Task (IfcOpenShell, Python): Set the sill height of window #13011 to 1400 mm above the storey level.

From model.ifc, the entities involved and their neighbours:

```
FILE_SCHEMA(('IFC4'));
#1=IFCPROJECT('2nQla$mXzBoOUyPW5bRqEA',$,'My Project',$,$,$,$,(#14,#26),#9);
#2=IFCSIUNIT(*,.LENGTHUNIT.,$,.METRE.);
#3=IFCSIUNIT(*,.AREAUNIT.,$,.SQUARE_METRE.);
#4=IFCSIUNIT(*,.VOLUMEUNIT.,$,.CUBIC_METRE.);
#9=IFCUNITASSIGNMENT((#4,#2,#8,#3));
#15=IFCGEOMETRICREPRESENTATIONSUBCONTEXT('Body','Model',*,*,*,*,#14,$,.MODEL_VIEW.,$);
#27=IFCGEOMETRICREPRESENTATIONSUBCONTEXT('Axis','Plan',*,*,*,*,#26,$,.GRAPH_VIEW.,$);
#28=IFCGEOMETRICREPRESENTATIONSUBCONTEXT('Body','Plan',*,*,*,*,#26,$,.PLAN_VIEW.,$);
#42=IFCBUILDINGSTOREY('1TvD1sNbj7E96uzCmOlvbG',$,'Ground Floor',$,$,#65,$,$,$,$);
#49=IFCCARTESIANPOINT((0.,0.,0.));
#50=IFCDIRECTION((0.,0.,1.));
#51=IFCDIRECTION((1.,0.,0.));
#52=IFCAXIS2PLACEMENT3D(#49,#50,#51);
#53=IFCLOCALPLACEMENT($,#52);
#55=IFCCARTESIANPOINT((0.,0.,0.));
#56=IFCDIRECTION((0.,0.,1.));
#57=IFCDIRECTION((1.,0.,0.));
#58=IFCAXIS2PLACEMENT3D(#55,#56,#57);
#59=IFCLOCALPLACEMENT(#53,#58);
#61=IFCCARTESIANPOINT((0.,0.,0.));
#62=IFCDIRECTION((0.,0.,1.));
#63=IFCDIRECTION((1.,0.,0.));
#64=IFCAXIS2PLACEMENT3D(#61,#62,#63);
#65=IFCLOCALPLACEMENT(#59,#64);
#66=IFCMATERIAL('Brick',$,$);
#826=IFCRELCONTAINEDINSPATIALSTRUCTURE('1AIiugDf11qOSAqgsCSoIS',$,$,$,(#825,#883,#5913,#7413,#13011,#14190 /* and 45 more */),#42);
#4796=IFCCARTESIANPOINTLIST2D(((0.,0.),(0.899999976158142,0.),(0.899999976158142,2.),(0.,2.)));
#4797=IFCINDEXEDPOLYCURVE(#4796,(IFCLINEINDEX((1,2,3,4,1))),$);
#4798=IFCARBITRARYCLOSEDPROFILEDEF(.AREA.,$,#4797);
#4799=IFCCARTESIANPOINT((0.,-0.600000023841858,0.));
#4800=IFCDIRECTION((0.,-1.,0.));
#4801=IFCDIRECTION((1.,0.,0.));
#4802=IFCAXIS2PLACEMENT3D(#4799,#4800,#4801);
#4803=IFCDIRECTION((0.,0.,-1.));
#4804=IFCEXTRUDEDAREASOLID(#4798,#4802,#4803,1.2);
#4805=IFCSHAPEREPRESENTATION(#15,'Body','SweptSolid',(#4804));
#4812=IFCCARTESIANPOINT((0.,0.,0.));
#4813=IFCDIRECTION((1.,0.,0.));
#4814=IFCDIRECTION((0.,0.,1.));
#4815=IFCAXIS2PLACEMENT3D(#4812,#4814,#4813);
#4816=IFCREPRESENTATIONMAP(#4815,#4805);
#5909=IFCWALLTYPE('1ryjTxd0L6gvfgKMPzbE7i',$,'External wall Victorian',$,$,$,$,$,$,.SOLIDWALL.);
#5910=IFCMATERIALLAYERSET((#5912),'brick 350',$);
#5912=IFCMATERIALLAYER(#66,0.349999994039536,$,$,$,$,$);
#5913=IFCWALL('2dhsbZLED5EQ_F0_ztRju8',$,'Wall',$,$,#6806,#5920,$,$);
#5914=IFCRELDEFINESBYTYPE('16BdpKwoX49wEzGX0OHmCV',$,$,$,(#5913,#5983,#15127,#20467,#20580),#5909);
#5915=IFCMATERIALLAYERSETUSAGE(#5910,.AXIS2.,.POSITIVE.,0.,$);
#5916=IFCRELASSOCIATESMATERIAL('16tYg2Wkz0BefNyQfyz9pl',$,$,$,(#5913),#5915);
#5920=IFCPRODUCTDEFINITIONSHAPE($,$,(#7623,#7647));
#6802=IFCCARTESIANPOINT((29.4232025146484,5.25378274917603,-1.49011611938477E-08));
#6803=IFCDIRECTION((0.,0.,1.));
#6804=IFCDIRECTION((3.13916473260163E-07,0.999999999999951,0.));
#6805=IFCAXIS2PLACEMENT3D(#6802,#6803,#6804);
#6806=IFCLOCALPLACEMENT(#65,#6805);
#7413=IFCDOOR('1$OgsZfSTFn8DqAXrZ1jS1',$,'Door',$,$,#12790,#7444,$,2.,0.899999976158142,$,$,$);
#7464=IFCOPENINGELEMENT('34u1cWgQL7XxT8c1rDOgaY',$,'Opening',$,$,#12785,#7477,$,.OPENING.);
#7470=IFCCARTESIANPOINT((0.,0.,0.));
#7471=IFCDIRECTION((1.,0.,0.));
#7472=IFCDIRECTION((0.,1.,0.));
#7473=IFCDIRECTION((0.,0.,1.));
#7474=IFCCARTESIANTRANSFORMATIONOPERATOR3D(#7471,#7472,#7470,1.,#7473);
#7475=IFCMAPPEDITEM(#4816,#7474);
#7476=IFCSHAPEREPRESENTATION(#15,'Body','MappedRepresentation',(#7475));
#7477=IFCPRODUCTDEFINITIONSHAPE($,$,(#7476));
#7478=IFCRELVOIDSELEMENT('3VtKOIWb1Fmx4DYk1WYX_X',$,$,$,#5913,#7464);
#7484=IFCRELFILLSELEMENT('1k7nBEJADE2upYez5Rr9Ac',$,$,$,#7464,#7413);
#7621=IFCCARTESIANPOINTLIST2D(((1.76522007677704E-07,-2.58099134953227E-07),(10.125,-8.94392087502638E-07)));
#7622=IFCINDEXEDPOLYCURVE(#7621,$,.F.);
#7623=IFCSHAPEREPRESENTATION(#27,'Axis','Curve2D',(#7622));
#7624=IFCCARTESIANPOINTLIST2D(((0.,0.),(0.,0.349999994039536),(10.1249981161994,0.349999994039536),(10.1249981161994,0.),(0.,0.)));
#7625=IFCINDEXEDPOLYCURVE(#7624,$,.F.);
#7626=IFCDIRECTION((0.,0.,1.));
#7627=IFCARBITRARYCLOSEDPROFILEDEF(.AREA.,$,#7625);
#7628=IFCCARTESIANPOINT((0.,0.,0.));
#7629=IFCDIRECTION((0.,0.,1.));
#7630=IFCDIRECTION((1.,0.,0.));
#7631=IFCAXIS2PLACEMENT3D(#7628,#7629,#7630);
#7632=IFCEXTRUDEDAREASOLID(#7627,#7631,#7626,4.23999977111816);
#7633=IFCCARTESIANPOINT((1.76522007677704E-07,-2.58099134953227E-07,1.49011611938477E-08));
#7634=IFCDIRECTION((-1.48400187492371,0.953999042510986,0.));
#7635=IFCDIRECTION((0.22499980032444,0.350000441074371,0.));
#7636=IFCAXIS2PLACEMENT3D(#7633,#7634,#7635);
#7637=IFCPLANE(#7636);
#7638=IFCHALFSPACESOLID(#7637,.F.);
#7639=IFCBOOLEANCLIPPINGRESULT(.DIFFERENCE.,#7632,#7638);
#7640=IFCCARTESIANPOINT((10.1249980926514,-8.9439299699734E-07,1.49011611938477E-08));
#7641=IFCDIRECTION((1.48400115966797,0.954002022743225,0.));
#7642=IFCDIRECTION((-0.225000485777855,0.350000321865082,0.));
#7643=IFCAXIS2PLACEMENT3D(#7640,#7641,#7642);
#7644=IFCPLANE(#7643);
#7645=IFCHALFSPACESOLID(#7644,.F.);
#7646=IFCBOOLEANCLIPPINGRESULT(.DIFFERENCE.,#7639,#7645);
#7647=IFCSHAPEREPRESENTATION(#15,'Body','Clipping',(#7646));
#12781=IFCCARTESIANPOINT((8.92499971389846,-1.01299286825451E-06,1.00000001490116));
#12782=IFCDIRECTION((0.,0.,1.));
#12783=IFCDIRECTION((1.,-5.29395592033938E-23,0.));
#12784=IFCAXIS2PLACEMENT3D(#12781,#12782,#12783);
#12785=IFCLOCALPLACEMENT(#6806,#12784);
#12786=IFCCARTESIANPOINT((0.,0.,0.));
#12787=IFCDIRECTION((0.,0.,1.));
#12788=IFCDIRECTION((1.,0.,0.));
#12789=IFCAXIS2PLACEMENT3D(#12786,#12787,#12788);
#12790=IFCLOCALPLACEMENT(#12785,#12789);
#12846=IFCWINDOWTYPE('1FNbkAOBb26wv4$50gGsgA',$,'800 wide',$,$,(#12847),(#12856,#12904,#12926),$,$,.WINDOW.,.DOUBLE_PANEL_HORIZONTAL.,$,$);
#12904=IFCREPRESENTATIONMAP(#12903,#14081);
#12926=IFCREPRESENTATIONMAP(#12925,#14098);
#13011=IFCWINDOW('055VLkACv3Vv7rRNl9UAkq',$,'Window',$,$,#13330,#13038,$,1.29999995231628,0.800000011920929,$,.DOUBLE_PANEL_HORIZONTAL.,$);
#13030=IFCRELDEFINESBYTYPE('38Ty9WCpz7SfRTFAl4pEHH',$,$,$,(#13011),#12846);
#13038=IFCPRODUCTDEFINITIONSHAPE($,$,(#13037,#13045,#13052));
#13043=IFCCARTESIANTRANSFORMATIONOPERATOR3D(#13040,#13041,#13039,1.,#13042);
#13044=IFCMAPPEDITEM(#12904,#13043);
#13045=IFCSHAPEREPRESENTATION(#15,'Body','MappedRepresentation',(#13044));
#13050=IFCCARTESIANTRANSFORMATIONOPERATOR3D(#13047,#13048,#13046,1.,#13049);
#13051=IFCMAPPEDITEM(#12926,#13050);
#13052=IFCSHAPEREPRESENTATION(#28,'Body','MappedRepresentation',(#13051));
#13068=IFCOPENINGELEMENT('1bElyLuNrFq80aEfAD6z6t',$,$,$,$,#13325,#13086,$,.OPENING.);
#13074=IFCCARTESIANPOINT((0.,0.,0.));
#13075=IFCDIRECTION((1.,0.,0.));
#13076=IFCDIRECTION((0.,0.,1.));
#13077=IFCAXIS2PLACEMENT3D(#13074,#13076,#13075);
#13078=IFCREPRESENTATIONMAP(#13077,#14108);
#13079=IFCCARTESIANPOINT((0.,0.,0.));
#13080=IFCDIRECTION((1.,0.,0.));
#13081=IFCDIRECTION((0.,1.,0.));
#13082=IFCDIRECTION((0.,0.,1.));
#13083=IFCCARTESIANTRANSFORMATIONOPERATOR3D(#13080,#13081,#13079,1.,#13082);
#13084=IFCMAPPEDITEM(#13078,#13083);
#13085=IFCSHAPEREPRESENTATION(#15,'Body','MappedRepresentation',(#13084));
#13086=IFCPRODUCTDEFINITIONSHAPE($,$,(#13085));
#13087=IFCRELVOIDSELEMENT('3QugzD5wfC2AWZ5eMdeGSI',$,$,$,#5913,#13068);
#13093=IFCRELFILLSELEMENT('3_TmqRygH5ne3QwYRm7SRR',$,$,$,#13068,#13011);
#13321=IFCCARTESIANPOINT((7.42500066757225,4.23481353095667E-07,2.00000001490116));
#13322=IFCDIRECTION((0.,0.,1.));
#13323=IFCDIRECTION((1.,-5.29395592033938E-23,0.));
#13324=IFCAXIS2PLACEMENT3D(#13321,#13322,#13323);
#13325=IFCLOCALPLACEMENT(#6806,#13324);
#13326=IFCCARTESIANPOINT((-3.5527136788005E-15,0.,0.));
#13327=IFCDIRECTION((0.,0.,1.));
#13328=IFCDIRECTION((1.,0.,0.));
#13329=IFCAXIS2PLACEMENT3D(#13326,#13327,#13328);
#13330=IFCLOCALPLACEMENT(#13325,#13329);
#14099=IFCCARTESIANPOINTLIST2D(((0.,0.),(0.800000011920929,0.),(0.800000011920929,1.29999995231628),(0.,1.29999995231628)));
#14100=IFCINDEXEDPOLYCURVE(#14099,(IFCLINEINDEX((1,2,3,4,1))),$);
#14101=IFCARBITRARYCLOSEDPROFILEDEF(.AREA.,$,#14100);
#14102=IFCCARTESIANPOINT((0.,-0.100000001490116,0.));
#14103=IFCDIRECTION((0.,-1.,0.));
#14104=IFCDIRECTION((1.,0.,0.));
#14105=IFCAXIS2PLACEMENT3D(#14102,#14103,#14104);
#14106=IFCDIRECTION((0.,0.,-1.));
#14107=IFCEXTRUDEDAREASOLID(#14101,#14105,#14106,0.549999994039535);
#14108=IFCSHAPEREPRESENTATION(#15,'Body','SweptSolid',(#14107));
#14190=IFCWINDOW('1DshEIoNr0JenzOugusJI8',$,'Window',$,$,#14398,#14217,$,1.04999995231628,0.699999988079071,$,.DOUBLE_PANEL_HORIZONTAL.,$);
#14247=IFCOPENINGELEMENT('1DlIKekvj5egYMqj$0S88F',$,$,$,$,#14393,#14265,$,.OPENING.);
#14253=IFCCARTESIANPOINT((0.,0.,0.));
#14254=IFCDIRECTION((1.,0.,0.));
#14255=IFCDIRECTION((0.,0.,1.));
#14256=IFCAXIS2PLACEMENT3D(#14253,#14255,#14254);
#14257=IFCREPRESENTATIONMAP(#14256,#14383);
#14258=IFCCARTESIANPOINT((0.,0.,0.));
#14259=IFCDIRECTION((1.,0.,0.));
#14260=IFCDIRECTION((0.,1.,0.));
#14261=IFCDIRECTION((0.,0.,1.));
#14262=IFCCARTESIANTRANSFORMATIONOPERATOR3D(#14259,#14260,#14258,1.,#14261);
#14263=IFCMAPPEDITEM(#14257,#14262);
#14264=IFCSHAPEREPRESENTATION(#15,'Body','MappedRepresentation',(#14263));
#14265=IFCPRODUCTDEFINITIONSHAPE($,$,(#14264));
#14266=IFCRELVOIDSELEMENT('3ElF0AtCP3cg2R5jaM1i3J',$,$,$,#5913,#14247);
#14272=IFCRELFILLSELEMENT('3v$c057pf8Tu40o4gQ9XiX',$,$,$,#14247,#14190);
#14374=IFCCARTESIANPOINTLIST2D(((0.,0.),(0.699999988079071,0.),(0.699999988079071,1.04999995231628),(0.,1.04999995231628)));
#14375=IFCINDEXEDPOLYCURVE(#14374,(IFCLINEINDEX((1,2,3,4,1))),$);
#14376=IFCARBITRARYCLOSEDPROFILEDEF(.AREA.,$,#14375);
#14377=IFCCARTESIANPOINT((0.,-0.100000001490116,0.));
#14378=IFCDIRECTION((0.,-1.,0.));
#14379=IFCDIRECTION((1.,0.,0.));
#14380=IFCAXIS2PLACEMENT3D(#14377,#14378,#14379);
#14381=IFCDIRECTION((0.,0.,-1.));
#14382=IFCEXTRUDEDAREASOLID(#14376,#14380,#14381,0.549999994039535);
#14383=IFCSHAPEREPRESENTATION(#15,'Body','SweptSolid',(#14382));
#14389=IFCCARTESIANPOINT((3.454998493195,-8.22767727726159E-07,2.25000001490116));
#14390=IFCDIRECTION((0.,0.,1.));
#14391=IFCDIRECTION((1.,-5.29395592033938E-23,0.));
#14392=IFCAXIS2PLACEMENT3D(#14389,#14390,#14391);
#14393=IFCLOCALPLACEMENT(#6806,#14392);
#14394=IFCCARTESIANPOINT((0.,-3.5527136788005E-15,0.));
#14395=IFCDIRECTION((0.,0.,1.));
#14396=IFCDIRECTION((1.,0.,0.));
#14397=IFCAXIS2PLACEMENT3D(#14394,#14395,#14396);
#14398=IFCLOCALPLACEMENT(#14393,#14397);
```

```python
import numpy as np
import ifcopenshell
import ifcopenshell.api.geometry
import ifcopenshell.geom
import ifcopenshell.util.element
import ifcopenshell.util.placement
import ifcopenshell.util.shape
import ifcopenshell.util.unit

model = ifcopenshell.open("model.ifc")
unit_scale = ifcopenshell.util.unit.calculate_unit_scale(model)

window = model.by_id(13011)
opening = window.FillsVoids[0].RelatingOpeningElement
storey = ifcopenshell.util.element.get_container(window, ifc_class="IfcBuildingStorey")
level = ifcopenshell.util.placement.get_local_placement(storey.ObjectPlacement)[2, 3]

# The opening's origin need not be at the sill, so measure its lowest point.
shape = ifcopenshell.geom.create_shape(ifcopenshell.geom.settings(), opening)
bottom = ifcopenshell.util.shape.get_shape_bottom_elevation(shape, shape.geometry) / unit_scale
dz = level + 1.4 - bottom

shift = np.array([0.0, 0.0, dz])
# The window is placed relative to its opening, so it follows when the opening moves.
matrix = ifcopenshell.util.placement.get_local_placement(opening.ObjectPlacement)
matrix[:3, 3] += shift
ifcopenshell.api.geometry.edit_object_placement(
    model, product=opening, matrix=matrix, is_si=False, should_transform_children=True
)

print(f"moved by {dz * unit_scale:+.3f} m")

model.write("model_updated.ifc")
```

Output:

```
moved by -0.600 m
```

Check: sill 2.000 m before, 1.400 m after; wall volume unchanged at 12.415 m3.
